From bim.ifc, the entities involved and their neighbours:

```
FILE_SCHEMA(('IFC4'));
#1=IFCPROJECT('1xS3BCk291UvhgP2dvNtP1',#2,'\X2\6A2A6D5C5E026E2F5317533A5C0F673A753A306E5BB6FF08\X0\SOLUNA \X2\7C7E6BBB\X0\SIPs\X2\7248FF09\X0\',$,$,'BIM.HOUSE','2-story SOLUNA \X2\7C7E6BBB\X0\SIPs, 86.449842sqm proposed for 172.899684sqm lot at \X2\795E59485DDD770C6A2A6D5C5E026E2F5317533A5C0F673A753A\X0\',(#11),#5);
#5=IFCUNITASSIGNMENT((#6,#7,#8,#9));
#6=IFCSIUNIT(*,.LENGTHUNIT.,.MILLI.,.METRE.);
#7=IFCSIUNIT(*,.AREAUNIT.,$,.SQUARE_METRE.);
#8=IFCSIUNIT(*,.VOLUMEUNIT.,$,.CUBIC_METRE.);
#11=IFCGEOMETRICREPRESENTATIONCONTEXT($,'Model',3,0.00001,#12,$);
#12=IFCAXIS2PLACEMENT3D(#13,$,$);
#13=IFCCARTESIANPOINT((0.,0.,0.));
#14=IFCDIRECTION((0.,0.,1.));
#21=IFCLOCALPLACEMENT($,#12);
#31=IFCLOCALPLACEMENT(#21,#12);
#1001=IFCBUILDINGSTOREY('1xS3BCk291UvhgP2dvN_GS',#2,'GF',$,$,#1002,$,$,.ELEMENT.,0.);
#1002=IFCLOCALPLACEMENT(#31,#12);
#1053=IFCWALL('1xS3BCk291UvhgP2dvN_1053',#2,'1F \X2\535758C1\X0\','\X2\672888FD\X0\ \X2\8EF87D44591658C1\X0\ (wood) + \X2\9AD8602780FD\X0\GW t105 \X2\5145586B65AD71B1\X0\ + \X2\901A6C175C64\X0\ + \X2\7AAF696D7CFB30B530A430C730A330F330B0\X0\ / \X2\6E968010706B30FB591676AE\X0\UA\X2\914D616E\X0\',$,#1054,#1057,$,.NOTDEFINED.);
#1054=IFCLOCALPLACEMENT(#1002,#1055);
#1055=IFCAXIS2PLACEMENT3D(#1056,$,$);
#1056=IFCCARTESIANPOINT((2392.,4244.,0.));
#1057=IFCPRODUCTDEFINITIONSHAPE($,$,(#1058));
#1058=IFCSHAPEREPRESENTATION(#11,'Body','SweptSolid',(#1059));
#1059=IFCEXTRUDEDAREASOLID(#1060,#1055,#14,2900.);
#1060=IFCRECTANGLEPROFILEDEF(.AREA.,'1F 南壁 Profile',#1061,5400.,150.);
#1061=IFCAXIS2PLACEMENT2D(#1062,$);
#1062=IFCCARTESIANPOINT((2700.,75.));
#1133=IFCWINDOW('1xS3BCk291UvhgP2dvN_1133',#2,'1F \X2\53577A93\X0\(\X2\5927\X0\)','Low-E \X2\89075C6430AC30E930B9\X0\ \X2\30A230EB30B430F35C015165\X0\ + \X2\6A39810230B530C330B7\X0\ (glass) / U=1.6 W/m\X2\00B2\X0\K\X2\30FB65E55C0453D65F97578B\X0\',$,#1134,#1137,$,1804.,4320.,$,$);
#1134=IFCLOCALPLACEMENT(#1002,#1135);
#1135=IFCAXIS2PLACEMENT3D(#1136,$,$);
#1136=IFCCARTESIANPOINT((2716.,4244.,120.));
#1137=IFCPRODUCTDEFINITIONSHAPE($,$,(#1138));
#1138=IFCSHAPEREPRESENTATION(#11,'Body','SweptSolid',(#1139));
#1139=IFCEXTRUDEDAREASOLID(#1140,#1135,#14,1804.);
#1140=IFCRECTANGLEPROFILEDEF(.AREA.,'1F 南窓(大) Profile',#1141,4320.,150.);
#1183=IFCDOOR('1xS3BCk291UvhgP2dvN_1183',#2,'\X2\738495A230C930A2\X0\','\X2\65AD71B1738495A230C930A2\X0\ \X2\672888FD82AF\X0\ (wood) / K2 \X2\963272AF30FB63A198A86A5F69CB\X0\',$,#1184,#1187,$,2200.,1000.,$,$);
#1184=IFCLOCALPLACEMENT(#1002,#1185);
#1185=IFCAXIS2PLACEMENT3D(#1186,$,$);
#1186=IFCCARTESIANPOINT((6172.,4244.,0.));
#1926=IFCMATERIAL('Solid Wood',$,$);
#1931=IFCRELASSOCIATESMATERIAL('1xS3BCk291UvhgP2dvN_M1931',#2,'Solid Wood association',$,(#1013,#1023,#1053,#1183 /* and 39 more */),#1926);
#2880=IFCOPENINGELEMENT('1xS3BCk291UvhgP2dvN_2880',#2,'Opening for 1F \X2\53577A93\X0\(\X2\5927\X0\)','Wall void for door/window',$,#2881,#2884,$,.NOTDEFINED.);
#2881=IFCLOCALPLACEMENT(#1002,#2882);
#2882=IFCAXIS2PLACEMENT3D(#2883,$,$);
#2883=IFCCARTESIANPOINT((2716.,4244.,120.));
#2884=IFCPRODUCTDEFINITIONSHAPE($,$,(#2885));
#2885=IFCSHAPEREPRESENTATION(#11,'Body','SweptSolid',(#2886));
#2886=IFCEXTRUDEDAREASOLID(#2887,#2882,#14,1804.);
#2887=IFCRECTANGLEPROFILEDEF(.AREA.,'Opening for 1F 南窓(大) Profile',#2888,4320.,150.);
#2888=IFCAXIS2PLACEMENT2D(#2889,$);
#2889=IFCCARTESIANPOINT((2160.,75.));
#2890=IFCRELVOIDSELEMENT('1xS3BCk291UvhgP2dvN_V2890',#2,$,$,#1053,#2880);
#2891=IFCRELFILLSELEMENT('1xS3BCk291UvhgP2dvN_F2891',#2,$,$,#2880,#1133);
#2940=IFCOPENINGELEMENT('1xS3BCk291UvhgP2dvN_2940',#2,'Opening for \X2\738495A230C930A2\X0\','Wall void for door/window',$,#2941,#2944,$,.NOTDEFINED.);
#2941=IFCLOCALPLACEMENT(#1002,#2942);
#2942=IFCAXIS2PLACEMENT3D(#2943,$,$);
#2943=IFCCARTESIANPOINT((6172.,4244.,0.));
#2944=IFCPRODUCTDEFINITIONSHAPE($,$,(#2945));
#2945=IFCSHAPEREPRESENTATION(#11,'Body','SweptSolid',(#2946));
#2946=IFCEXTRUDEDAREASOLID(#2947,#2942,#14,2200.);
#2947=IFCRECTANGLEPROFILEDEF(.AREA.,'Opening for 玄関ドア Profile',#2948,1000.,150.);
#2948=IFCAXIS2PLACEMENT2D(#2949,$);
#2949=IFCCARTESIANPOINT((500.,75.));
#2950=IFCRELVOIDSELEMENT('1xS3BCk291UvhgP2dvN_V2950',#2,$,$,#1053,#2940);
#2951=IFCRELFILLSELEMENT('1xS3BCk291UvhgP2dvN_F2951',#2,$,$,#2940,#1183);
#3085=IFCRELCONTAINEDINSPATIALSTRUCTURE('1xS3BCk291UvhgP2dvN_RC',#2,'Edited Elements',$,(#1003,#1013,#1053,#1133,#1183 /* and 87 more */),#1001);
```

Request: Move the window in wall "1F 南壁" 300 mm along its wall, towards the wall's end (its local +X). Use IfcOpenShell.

```python
import ifcopenshell
import ifcopenshell.api.geometry
import ifcopenshell.util.placement
import ifcopenshell.util.unit

model = ifcopenshell.open("bim.ifc")
unit_scale = ifcopenshell.util.unit.calculate_unit_scale(model)

window = model.by_guid("1xS3BCk291UvhgP2dvN_1133")
opening = window.FillsVoids[0].RelatingOpeningElement
wall = opening.VoidsElements[0].RelatingBuildingElement

wall_matrix = ifcopenshell.util.placement.get_local_placement(wall.ObjectPlacement)
shift = wall_matrix[:3, 0] * 0.3 / unit_scale
before = ifcopenshell.util.placement.get_local_placement(window.ObjectPlacement)[:3, 3].copy()

# The window is not placed relative to its opening, so move both.
for product in (opening, window):
    matrix = ifcopenshell.util.placement.get_local_placement(product.ObjectPlacement)
    matrix[:3, 3] += shift
    ifcopenshell.api.geometry.edit_object_placement(model, product=product, matrix=matrix, is_si=False)

after = ifcopenshell.util.placement.get_local_placement(window.ObjectPlacement)[:3, 3]
print("window moved by", (after - before).round(3) + 0.0)

model.write("bim_updated.ifc")
```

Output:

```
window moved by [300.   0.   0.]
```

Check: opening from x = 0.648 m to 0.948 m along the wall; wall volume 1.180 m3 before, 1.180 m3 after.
